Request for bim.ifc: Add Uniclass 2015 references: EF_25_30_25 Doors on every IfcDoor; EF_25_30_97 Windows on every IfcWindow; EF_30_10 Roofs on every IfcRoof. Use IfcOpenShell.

First a look at what the model holds.

```python
import ifcopenshell

model = ifcopenshell.open("bim.ifc")
print(model.schema)
print("classifications:", [c.Name for c in model.by_type("IfcClassification")])
for ifc_class in ("IfcDoor", "IfcRoof", "IfcStair", "IfcWall", "IfcWindow"):
    print(ifc_class, len(model.by_type(ifc_class)))
```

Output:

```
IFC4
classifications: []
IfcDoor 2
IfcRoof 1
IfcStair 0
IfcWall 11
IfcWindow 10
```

```python
import ifcopenshell
import ifcopenshell.api.classification

model = ifcopenshell.open("bim.ifc")

system = ifcopenshell.api.classification.add_classification(model, classification="Uniclass 2015")

codes = {
    "IfcDoor": ("EF_25_30_25", "Doors"),
    "IfcWindow": ("EF_25_30_97", "Windows"),
    "IfcRoof": ("EF_30_10", "Roofs"),
}
for ifc_class, (code, name) in codes.items():
    products = model.by_type(ifc_class)
    ifcopenshell.api.classification.add_reference(
        model, products=products, classification=system, identification=code, name=name
    )
    print(code, len(products))

model.write("bim-out.ifc")
```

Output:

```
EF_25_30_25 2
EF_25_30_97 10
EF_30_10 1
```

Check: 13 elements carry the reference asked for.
